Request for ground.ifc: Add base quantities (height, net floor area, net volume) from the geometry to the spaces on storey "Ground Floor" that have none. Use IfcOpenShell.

First a look at what the model holds.

```python
import ifcopenshell
import ifcopenshell.util.element
import ifcopenshell.util.unit

model = ifcopenshell.open("ground.ifc")
print(model.schema)
for unit_type in ("LENGTHUNIT", "AREAUNIT", "VOLUMEUNIT"):
    print(unit_type, ifcopenshell.util.unit.calculate_unit_scale(model, unit_type))
storey = next(s for s in model.by_type("IfcBuildingStorey") if s.Name == "Ground Floor")
spaces = [e for e in ifcopenshell.util.element.get_decomposition(storey) if e.is_a("IfcSpace")]
for e in sorted(spaces, key=lambda e: e.id()):
    print(e.id(), e.is_a(), e.Name, list(ifcopenshell.util.element.get_psets(e, qtos_only=True)), sep=" | ")
```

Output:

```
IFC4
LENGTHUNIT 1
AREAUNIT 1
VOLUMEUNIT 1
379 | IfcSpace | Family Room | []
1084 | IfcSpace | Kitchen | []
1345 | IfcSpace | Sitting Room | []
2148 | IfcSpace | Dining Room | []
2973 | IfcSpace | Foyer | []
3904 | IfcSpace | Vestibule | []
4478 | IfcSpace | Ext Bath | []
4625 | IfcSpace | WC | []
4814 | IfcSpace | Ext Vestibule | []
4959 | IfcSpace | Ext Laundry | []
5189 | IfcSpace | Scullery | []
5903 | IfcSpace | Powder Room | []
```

```python
import ifcopenshell
import ifcopenshell.api.pset
import ifcopenshell.geom
import ifcopenshell.util.element
import ifcopenshell.util.shape
import ifcopenshell.util.unit

model = ifcopenshell.open("ground.ifc")
unit_scale = ifcopenshell.util.unit.calculate_unit_scale(model)
area_scale = ifcopenshell.util.unit.calculate_unit_scale(model, "AREAUNIT")
volume_scale = ifcopenshell.util.unit.calculate_unit_scale(model, "VOLUMEUNIT")
settings = ifcopenshell.geom.settings()

storey = next(s for s in model.by_type("IfcBuildingStorey") if s.Name == "Ground Floor")
spaces = [e for e in ifcopenshell.util.element.get_decomposition(storey) if e.is_a("IfcSpace")]

for e in sorted(spaces, key=lambda e: e.id()):
    if ifcopenshell.util.element.get_psets(e, qtos_only=True, should_inherit=False):
        continue
    # Geometry comes back in metres, in the element's own axes.
    shape = ifcopenshell.geom.create_shape(settings, e)
    values = {
        "Height": ifcopenshell.util.shape.get_z(shape.geometry) / unit_scale,
        "NetFloorArea": ifcopenshell.util.shape.get_footprint_area(shape.geometry) / area_scale,
        "NetVolume": ifcopenshell.util.shape.get_volume(shape.geometry) / volume_scale,
    }
    qto = ifcopenshell.api.pset.add_qto(model, product=e, name="Qto_SpaceBaseQuantities")
    ifcopenshell.api.pset.edit_qto(model, qto=qto, properties=values)
    print(e.id(), {k: round(v, 3) for k, v in values.items()})

model.write("ground-out.ifc")
```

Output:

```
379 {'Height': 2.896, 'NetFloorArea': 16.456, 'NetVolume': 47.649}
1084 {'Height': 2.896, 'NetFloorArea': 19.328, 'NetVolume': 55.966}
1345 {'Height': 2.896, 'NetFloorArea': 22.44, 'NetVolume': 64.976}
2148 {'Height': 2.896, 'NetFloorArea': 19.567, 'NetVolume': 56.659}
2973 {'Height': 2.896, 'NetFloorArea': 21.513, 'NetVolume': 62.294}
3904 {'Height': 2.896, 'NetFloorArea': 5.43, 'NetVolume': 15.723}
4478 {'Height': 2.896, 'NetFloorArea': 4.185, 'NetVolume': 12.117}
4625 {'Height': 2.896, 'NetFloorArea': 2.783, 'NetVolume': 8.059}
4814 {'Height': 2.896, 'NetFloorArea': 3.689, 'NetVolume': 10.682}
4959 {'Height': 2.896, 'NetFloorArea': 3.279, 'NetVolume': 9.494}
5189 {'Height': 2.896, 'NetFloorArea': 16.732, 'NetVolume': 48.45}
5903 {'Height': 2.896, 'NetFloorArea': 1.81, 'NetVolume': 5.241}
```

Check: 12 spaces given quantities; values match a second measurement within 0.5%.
